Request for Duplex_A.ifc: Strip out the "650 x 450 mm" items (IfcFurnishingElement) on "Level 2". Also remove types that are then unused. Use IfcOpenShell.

First a look at what the model holds.

```python
import ifcopenshell
import ifcopenshell.util.element

model = ifcopenshell.open("Duplex_A.ifc")
print(model.schema)
storey = next(s for s in model.by_type("IfcBuildingStorey") if s.Name == "Level 2")
furniture = [e for e in ifcopenshell.util.element.get_decomposition(storey) if e.is_a("IfcFurnishingElement")]
seen = {}
for e in furniture:
    element_type = ifcopenshell.util.element.get_type(e)
    name = element_type.Name if element_type not in (None, e) else None
    seen[name] = seen.get(name, 0) + 1
for name, count in sorted(seen.items(), key=str):
    print(count, "x", name)
```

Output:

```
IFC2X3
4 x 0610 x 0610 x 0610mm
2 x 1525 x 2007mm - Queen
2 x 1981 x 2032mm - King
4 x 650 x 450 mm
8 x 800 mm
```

```python
import ifcopenshell
import ifcopenshell.api.root
import ifcopenshell.util.element

model = ifcopenshell.open("Duplex_A.ifc")

storey = next(s for s in model.by_type("IfcBuildingStorey") if s.Name == "Level 2")
furniture = [e for e in ifcopenshell.util.element.get_decomposition(storey) if e.is_a("IfcFurnishingElement")]
targets = [e for e in furniture if (t := ifcopenshell.util.element.get_type(e)) not in (None, e) and t.Name == "650 x 450 mm"]
types = {ifcopenshell.util.element.get_type(e) for e in targets} - {None, *targets}

for e in targets:
    ifcopenshell.api.root.remove_product(model, product=e)
print(len(targets), "removed")

unused = [t for t in types if not ifcopenshell.util.element.get_types(t)]
for t in unused:
    ifcopenshell.api.root.remove_product(model, product=t)
print(len(unused), "unused types removed")

model.write("Duplex_A-out.ifc")
```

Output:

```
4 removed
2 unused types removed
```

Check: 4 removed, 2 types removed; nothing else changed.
